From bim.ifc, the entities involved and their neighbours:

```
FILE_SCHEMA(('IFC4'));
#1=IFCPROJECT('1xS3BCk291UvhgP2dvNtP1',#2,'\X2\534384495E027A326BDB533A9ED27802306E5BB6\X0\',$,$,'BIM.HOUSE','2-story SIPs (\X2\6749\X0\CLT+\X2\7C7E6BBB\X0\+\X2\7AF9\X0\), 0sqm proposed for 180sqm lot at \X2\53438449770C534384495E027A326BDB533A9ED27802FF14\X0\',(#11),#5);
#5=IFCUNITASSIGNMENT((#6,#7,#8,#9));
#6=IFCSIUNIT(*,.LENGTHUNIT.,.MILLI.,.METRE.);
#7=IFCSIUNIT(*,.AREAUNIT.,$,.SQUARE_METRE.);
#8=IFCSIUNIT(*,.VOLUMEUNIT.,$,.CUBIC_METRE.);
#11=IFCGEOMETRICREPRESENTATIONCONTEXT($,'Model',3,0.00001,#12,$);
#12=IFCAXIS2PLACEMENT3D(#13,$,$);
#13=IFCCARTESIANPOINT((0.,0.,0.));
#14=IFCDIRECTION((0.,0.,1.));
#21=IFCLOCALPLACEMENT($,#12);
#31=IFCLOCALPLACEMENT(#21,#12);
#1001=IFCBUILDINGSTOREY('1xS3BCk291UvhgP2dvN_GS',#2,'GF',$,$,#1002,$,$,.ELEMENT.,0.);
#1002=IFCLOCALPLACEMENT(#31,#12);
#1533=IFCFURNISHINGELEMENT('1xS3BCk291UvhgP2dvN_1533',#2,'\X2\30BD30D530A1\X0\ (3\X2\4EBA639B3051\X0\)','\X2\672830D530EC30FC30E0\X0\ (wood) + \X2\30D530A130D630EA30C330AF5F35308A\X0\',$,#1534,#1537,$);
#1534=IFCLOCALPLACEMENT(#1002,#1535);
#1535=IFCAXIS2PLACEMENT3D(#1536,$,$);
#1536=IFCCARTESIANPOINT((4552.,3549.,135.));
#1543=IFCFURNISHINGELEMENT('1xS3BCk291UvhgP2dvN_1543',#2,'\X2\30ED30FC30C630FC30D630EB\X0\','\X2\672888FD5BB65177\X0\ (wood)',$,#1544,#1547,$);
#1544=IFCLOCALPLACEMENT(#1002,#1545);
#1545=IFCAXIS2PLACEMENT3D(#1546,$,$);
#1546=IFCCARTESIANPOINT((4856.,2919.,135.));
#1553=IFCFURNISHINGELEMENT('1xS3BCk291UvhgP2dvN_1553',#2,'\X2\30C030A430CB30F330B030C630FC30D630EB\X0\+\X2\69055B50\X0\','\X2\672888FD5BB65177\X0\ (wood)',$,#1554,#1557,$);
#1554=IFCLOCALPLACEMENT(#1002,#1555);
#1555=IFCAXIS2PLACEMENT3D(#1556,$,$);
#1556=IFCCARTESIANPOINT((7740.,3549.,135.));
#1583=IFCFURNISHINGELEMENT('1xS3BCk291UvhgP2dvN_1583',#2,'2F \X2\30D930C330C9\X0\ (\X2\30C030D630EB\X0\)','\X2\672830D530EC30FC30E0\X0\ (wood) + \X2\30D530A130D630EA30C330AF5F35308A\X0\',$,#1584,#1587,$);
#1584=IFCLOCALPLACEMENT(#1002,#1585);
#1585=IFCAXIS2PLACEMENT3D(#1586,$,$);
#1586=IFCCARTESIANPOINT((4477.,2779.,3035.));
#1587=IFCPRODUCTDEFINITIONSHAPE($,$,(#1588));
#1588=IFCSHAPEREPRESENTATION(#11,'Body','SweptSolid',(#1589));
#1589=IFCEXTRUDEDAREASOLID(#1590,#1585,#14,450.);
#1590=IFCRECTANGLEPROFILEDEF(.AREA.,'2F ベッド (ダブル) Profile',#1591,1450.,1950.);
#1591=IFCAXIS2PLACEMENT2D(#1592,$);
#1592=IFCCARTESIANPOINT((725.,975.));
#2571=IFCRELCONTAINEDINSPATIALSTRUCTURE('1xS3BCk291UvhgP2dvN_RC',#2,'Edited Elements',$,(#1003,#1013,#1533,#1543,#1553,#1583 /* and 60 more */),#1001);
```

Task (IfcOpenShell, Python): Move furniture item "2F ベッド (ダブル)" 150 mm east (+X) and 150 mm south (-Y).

```python
import ifcopenshell
import ifcopenshell.api.geometry
import ifcopenshell.util.placement
import ifcopenshell.util.unit

model = ifcopenshell.open("bim.ifc")
unit_scale = ifcopenshell.util.unit.calculate_unit_scale(model)

item = model.by_id(1583)
matrix = ifcopenshell.util.placement.get_local_placement(item.ObjectPlacement)
matrix[0, 3] += 0.15 / unit_scale
matrix[1, 3] -= 0.15 / unit_scale
ifcopenshell.api.geometry.edit_object_placement(model, product=item, matrix=matrix, is_si=False)

print(ifcopenshell.util.placement.get_local_placement(item.ObjectPlacement).round(3) + 0.0)

model.write("bim_edited.ifc")
```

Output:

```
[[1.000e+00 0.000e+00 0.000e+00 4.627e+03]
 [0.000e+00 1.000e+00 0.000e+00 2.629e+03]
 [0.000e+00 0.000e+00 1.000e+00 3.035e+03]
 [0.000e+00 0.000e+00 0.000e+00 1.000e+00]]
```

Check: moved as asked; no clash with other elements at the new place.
